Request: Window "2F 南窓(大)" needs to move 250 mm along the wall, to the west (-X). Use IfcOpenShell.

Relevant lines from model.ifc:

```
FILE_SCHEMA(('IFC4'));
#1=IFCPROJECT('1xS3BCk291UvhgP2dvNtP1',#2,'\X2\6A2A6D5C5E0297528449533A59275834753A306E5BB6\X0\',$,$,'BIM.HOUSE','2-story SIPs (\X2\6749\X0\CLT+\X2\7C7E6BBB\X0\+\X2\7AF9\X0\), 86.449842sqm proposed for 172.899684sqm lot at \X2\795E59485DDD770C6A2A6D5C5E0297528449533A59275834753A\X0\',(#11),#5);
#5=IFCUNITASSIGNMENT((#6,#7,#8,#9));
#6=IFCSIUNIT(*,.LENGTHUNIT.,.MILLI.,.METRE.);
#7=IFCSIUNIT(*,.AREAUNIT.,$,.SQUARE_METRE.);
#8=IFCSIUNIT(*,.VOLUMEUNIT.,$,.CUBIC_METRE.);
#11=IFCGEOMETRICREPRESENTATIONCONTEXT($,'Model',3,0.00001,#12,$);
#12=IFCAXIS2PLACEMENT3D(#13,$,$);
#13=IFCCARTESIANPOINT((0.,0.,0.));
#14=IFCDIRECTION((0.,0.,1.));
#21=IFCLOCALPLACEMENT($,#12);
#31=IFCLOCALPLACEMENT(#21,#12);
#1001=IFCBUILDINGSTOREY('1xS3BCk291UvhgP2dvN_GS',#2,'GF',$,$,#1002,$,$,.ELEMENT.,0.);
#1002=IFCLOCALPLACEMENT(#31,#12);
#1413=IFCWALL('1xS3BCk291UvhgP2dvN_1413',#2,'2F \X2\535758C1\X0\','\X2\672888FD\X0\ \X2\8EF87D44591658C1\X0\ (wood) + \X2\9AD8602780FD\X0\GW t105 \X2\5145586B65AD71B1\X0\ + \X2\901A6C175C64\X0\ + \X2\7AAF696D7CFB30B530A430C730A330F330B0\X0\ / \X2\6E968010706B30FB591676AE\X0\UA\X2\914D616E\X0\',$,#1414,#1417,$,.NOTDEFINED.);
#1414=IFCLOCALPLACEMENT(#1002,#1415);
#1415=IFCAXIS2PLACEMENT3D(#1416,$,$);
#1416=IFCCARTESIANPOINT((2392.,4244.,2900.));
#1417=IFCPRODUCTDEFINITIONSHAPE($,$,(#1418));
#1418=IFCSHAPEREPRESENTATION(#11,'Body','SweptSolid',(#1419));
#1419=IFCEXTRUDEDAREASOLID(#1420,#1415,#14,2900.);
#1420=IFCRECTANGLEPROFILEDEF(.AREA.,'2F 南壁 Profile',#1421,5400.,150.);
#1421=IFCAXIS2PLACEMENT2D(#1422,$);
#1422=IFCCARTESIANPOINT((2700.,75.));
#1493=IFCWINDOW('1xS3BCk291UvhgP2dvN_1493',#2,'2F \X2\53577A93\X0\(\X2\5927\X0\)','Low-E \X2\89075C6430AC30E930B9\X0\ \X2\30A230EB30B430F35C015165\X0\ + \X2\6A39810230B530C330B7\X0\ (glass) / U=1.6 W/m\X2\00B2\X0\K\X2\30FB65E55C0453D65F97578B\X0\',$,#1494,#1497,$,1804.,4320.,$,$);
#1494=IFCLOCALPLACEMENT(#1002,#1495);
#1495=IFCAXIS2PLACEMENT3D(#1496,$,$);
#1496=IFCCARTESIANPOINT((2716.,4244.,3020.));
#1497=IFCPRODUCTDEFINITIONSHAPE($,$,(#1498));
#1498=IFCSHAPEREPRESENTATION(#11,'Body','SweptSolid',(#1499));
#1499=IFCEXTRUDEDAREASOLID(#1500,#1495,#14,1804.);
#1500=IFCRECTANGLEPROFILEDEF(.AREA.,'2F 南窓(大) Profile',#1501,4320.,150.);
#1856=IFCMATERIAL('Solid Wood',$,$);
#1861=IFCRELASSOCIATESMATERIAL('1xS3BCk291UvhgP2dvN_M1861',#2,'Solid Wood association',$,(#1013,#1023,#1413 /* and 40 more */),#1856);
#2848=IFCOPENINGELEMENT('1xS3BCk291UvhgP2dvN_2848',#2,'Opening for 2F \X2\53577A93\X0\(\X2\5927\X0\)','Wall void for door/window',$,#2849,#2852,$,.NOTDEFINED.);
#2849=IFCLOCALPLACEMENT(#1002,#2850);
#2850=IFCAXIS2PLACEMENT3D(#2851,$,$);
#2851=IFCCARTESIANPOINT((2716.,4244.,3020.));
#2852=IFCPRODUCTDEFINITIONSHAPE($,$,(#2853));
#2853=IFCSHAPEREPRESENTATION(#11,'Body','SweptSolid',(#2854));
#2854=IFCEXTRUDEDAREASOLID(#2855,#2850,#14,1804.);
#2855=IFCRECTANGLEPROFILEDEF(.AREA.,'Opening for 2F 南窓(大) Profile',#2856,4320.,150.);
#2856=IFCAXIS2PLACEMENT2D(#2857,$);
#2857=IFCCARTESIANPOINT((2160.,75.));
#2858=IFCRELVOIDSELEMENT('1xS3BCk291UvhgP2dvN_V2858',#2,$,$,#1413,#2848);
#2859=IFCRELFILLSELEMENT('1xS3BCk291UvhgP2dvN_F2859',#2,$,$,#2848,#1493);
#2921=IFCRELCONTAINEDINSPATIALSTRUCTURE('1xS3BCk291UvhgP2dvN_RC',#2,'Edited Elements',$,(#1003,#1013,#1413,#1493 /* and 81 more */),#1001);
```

```python
import ifcopenshell
import ifcopenshell.api.geometry
import ifcopenshell.util.placement
import ifcopenshell.util.unit

model = ifcopenshell.open("model.ifc")
unit_scale = ifcopenshell.util.unit.calculate_unit_scale(model)

window = model.by_guid("1xS3BCk291UvhgP2dvN_1493")
opening = window.FillsVoids[0].RelatingOpeningElement
wall = opening.VoidsElements[0].RelatingBuildingElement

wall_matrix = ifcopenshell.util.placement.get_local_placement(wall.ObjectPlacement)
shift = wall_matrix[:3, 0] * -0.25 / unit_scale
before = ifcopenshell.util.placement.get_local_placement(window.ObjectPlacement)[:3, 3].copy()

# The window is not placed relative to its opening, so move both.
for product in (opening, window):
    matrix = ifcopenshell.util.placement.get_local_placement(product.ObjectPlacement)
    matrix[:3, 3] += shift
    ifcopenshell.api.geometry.edit_object_placement(model, product=product, matrix=matrix, is_si=False)

after = ifcopenshell.util.placement.get_local_placement(window.ObjectPlacement)[:3, 3]
print("window moved by", (after - before).round(3) + 0.0)

model.write("model-out.ifc")
```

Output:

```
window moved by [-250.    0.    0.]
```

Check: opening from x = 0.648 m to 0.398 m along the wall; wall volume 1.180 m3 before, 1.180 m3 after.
